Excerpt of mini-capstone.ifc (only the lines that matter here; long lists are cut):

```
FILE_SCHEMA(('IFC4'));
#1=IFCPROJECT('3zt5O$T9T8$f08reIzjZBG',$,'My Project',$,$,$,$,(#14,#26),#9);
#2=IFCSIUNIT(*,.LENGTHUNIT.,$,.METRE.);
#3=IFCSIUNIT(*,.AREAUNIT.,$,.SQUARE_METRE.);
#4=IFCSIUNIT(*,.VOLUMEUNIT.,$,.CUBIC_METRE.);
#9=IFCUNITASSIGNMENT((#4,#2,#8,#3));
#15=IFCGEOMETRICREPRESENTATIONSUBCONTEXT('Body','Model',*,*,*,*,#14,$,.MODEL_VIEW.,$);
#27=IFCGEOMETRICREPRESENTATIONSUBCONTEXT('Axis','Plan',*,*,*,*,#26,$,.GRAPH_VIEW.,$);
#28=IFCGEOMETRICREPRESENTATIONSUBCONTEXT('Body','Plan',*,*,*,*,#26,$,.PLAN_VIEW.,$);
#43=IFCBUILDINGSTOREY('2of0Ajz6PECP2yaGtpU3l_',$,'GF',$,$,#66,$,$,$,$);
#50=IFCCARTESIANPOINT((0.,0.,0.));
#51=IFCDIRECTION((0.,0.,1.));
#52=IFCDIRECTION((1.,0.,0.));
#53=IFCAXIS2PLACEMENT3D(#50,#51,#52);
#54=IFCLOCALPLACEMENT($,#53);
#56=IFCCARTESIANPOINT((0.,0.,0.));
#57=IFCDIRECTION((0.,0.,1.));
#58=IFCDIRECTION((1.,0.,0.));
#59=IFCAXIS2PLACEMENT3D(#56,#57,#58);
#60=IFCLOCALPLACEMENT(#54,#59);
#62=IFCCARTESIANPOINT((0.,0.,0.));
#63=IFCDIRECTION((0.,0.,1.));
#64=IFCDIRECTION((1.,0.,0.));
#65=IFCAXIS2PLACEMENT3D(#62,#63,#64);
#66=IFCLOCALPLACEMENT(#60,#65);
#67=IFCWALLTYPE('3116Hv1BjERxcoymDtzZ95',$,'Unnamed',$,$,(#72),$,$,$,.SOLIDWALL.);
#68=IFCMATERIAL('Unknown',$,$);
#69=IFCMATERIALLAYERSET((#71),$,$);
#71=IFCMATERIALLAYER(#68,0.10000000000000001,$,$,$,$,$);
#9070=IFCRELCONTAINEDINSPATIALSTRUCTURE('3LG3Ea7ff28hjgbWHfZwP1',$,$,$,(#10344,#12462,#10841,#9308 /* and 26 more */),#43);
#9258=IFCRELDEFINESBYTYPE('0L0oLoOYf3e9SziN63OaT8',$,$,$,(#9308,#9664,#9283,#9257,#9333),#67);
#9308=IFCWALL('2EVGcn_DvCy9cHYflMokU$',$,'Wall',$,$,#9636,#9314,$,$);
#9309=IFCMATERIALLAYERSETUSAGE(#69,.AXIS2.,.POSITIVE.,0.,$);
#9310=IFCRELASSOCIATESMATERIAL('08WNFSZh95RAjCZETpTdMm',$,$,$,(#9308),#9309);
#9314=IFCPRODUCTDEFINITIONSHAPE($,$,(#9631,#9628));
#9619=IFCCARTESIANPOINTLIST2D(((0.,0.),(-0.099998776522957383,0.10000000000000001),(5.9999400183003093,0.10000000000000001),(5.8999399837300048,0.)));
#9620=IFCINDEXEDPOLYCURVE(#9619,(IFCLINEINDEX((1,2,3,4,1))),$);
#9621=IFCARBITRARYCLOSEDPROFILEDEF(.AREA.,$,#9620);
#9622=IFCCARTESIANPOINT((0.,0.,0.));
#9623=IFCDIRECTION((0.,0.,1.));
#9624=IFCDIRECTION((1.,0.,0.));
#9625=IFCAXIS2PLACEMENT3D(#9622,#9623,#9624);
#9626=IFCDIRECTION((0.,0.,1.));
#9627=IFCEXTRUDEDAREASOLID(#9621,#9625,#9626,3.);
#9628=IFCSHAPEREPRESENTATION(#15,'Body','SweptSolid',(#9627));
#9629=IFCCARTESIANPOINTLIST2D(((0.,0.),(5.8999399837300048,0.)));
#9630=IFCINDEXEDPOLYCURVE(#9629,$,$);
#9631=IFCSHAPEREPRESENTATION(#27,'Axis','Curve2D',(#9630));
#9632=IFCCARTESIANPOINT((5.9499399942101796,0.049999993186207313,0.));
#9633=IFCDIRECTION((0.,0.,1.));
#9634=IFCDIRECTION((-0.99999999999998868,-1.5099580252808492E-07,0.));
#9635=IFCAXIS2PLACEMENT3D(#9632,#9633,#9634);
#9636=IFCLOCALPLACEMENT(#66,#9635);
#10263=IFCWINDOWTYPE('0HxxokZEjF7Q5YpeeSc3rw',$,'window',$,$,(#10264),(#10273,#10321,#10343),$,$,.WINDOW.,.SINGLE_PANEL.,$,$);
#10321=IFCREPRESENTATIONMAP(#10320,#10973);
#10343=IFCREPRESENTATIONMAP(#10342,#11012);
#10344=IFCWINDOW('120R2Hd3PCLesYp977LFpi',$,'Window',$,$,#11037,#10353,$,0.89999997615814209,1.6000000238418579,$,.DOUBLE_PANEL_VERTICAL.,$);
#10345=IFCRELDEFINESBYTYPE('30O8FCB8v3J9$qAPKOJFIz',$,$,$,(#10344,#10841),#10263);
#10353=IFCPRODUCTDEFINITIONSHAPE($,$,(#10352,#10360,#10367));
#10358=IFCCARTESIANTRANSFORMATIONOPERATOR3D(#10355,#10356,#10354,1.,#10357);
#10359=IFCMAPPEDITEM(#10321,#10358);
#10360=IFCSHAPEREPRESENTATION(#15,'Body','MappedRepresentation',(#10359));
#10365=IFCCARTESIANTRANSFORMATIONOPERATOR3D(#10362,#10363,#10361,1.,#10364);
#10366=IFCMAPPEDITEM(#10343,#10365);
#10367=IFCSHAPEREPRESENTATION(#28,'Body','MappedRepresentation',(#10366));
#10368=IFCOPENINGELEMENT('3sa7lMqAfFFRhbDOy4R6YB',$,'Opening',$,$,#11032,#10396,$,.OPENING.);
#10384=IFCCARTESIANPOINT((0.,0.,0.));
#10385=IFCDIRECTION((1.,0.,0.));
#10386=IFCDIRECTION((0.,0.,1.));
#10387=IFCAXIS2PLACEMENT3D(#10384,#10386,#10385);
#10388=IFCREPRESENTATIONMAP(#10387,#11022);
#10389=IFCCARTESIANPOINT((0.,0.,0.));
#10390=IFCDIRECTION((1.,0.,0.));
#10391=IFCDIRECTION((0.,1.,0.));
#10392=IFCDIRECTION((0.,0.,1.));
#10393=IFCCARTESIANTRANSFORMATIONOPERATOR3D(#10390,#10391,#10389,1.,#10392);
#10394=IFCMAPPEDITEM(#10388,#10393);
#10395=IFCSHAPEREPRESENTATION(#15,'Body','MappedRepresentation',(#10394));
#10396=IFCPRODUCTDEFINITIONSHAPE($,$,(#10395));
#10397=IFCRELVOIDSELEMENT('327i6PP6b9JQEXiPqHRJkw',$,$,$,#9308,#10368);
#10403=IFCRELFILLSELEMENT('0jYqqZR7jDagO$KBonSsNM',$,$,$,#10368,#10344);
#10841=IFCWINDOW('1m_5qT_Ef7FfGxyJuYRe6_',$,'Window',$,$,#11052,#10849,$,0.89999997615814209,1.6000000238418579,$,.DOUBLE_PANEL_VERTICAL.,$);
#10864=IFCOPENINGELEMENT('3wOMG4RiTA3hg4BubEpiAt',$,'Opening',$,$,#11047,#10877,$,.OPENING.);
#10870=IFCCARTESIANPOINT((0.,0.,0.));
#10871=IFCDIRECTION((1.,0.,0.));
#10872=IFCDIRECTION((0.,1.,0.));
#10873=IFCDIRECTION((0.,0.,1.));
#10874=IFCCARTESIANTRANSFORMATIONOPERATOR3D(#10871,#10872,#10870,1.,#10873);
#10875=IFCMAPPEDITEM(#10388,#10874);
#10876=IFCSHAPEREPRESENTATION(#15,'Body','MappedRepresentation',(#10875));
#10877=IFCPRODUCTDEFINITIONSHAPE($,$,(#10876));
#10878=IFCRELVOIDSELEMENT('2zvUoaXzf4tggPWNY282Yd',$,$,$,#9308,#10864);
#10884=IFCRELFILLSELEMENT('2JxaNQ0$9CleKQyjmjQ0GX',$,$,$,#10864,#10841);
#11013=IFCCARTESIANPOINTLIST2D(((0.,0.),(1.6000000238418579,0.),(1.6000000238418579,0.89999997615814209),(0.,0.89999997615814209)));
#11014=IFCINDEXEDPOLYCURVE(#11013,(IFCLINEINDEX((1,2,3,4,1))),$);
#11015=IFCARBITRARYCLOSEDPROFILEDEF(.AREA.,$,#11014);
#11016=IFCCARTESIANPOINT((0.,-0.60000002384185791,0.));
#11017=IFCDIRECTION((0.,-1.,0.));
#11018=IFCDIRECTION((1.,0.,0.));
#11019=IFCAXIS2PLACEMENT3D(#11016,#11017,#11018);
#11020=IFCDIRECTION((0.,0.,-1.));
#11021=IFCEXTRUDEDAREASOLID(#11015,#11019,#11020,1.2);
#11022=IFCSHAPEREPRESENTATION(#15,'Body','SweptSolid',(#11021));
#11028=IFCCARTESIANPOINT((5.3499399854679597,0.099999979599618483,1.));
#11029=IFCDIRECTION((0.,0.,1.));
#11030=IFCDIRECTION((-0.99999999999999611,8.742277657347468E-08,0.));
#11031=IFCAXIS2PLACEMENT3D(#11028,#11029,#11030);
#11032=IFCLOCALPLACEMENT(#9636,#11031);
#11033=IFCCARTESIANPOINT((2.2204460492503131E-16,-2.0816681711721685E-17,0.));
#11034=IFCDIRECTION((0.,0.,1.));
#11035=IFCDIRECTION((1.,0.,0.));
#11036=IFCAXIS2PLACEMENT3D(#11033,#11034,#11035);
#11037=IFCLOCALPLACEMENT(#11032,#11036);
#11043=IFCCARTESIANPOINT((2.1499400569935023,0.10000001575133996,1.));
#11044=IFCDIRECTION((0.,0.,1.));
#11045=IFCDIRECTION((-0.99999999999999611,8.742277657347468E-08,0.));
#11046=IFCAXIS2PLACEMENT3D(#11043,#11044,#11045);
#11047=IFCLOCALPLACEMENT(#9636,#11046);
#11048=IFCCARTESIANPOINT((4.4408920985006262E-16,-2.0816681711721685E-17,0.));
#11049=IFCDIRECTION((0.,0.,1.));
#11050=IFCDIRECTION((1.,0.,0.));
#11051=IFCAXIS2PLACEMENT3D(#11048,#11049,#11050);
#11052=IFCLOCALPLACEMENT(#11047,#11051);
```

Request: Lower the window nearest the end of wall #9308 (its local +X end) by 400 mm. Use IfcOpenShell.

```python
import numpy as np
import ifcopenshell
import ifcopenshell.api.geometry
import ifcopenshell.util.placement
import ifcopenshell.util.unit

model = ifcopenshell.open("mini-capstone.ifc")
unit_scale = ifcopenshell.util.unit.calculate_unit_scale(model)

window = model.by_guid("120R2Hd3PCLesYp977LFpi")
opening = window.FillsVoids[0].RelatingOpeningElement
dz = -0.4 / unit_scale

shift = np.array([0.0, 0.0, dz])
# The window is placed relative to its opening, so it follows when the opening moves.
matrix = ifcopenshell.util.placement.get_local_placement(opening.ObjectPlacement)
matrix[:3, 3] += shift
ifcopenshell.api.geometry.edit_object_placement(
    model, product=opening, matrix=matrix, is_si=False, should_transform_children=True
)

print(f"moved by {dz * unit_scale:+.3f} m")

model.write("mini-capstone_edited.ifc")
```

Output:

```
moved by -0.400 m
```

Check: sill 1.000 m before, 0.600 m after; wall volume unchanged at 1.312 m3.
